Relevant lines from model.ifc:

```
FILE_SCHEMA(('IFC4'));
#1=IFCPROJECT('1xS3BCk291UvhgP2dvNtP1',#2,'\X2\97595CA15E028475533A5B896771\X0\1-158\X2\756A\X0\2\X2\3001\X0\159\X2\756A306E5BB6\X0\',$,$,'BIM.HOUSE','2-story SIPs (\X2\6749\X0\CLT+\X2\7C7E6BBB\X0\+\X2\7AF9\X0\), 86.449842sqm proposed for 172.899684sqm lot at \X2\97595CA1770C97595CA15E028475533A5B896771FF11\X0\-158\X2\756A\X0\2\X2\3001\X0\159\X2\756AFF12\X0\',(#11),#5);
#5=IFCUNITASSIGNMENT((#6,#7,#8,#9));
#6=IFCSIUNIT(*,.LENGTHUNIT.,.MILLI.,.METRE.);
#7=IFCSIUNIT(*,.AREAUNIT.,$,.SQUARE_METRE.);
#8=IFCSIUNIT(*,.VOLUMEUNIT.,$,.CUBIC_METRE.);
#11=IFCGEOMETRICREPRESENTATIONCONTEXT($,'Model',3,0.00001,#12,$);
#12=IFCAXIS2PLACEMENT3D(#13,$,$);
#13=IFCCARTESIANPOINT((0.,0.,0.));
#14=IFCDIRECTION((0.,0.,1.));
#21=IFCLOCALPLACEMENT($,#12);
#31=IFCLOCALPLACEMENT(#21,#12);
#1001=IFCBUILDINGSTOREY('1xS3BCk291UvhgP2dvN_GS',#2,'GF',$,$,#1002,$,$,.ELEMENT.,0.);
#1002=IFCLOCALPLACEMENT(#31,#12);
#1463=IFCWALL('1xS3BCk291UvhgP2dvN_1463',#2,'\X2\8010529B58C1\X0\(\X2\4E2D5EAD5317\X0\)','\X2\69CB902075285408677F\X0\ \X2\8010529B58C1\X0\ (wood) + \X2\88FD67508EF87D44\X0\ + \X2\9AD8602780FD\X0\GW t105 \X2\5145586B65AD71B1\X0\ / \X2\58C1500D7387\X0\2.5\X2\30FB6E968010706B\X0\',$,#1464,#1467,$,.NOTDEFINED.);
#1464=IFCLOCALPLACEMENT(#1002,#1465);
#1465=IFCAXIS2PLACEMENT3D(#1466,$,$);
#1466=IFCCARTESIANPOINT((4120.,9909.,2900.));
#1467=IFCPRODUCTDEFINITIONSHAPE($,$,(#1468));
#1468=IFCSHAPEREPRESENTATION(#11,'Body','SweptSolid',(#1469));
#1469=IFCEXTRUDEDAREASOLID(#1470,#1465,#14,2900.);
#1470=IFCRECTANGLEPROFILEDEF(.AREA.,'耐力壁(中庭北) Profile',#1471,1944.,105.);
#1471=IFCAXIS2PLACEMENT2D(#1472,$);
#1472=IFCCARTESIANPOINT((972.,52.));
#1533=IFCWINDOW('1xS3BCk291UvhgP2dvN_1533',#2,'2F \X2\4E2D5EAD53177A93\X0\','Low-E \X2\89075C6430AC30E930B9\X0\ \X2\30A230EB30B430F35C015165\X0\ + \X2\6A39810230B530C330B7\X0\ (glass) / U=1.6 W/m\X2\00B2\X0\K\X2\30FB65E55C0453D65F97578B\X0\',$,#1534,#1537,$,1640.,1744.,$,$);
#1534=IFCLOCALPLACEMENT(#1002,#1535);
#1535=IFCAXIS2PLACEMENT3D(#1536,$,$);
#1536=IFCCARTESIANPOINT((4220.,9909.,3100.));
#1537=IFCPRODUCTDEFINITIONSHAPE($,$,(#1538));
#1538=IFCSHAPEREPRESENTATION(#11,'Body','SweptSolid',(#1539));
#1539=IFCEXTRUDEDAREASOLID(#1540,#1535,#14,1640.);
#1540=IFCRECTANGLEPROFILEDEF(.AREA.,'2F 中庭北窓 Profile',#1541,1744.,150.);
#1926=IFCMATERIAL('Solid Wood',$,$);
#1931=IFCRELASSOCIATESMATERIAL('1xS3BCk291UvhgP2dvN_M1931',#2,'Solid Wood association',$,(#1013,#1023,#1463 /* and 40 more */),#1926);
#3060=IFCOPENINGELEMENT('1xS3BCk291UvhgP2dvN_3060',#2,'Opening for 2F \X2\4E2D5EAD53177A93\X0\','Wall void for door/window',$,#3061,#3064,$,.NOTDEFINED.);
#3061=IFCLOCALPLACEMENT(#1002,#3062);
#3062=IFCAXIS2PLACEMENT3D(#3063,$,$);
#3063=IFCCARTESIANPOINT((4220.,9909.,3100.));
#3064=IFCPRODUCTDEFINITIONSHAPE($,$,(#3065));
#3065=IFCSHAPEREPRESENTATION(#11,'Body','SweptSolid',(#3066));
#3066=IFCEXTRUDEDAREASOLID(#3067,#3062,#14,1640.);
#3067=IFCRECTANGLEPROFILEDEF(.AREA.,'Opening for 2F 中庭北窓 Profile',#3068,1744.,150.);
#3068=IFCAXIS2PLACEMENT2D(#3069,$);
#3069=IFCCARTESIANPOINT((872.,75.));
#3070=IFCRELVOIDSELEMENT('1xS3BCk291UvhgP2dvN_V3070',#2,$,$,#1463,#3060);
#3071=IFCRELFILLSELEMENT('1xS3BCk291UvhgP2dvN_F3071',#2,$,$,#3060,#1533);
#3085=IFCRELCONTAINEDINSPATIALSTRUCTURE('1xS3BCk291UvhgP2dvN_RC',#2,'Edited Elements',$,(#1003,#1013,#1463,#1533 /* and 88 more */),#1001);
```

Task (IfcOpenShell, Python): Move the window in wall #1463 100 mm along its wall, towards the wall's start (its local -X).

```python
import ifcopenshell
import ifcopenshell.api.geometry
import ifcopenshell.util.placement
import ifcopenshell.util.unit

model = ifcopenshell.open("model.ifc")
unit_scale = ifcopenshell.util.unit.calculate_unit_scale(model)

window = model.by_guid("1xS3BCk291UvhgP2dvN_1533")
opening = window.FillsVoids[0].RelatingOpeningElement
wall = opening.VoidsElements[0].RelatingBuildingElement

wall_matrix = ifcopenshell.util.placement.get_local_placement(wall.ObjectPlacement)
shift = wall_matrix[:3, 0] * -0.1 / unit_scale
before = ifcopenshell.util.placement.get_local_placement(window.ObjectPlacement)[:3, 3].copy()

# The window is not placed relative to its opening, so move both.
for product in (opening, window):
    matrix = ifcopenshell.util.placement.get_local_placement(product.ObjectPlacement)
    matrix[:3, 3] += shift
    ifcopenshell.api.geometry.edit_object_placement(model, product=product, matrix=matrix, is_si=False)

after = ifcopenshell.util.placement.get_local_placement(window.ObjectPlacement)[:3, 3]
print("window moved by", (after - before).round(3) + 0.0)

model.write("model_edited.ifc")
```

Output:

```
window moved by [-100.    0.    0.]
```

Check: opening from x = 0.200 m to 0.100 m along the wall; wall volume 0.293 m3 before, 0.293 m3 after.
